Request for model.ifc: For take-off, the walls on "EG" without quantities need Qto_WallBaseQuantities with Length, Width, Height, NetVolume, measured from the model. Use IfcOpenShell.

First a look at what the model holds.

```python
import ifcopenshell
import ifcopenshell.util.element
import ifcopenshell.util.unit

model = ifcopenshell.open("model.ifc")
print(model.schema)
for unit_type in ("LENGTHUNIT", "AREAUNIT", "VOLUMEUNIT"):
    print(unit_type, ifcopenshell.util.unit.calculate_unit_scale(model, unit_type))
storey = next(s for s in model.by_type("IfcBuildingStorey") if s.Name == "EG")
walls = [e for e in ifcopenshell.util.element.get_decomposition(storey) if e.is_a("IfcWall")]
for e in sorted(walls, key=lambda e: e.id()):
    print(e.id(), e.is_a(), e.Name, list(ifcopenshell.util.element.get_psets(e, qtos_only=True)), sep=" | ")
```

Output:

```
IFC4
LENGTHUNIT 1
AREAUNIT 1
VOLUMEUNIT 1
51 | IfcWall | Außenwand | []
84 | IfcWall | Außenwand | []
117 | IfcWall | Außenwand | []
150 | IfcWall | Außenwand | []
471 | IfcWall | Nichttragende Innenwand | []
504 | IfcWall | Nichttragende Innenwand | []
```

```python
import ifcopenshell
import ifcopenshell.api.pset
import ifcopenshell.geom
import ifcopenshell.util.element
import ifcopenshell.util.shape
import ifcopenshell.util.unit

model = ifcopenshell.open("model.ifc")
unit_scale = ifcopenshell.util.unit.calculate_unit_scale(model)
volume_scale = ifcopenshell.util.unit.calculate_unit_scale(model, "VOLUMEUNIT")
settings = ifcopenshell.geom.settings()

storey = next(s for s in model.by_type("IfcBuildingStorey") if s.Name == "EG")
walls = [e for e in ifcopenshell.util.element.get_decomposition(storey) if e.is_a("IfcWall")]

for e in sorted(walls, key=lambda e: e.id()):
    if ifcopenshell.util.element.get_psets(e, qtos_only=True, should_inherit=False):
        continue
    # Geometry comes back in metres, in the element's own axes.
    shape = ifcopenshell.geom.create_shape(settings, e)
    values = {
        "Length": ifcopenshell.util.shape.get_x(shape.geometry) / unit_scale,
        "Width": ifcopenshell.util.shape.get_y(shape.geometry) / unit_scale,
        "Height": ifcopenshell.util.shape.get_z(shape.geometry) / unit_scale,
        "NetVolume": ifcopenshell.util.shape.get_volume(shape.geometry) / volume_scale,
    }
    qto = ifcopenshell.api.pset.add_qto(model, product=e, name="Qto_WallBaseQuantities")
    ifcopenshell.api.pset.edit_qto(model, qto=qto, properties=values)
    print(e.id(), {k: round(v, 3) for k, v in values.items()})

model.write("model_edited.ifc")
```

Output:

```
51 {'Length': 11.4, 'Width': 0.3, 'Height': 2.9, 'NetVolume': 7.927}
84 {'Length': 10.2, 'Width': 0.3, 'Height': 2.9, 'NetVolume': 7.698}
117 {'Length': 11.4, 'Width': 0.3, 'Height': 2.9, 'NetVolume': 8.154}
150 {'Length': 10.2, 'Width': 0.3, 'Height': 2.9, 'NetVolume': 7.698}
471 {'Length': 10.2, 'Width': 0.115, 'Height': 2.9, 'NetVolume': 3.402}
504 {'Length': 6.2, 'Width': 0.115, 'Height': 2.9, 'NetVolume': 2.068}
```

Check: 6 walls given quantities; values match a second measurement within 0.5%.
